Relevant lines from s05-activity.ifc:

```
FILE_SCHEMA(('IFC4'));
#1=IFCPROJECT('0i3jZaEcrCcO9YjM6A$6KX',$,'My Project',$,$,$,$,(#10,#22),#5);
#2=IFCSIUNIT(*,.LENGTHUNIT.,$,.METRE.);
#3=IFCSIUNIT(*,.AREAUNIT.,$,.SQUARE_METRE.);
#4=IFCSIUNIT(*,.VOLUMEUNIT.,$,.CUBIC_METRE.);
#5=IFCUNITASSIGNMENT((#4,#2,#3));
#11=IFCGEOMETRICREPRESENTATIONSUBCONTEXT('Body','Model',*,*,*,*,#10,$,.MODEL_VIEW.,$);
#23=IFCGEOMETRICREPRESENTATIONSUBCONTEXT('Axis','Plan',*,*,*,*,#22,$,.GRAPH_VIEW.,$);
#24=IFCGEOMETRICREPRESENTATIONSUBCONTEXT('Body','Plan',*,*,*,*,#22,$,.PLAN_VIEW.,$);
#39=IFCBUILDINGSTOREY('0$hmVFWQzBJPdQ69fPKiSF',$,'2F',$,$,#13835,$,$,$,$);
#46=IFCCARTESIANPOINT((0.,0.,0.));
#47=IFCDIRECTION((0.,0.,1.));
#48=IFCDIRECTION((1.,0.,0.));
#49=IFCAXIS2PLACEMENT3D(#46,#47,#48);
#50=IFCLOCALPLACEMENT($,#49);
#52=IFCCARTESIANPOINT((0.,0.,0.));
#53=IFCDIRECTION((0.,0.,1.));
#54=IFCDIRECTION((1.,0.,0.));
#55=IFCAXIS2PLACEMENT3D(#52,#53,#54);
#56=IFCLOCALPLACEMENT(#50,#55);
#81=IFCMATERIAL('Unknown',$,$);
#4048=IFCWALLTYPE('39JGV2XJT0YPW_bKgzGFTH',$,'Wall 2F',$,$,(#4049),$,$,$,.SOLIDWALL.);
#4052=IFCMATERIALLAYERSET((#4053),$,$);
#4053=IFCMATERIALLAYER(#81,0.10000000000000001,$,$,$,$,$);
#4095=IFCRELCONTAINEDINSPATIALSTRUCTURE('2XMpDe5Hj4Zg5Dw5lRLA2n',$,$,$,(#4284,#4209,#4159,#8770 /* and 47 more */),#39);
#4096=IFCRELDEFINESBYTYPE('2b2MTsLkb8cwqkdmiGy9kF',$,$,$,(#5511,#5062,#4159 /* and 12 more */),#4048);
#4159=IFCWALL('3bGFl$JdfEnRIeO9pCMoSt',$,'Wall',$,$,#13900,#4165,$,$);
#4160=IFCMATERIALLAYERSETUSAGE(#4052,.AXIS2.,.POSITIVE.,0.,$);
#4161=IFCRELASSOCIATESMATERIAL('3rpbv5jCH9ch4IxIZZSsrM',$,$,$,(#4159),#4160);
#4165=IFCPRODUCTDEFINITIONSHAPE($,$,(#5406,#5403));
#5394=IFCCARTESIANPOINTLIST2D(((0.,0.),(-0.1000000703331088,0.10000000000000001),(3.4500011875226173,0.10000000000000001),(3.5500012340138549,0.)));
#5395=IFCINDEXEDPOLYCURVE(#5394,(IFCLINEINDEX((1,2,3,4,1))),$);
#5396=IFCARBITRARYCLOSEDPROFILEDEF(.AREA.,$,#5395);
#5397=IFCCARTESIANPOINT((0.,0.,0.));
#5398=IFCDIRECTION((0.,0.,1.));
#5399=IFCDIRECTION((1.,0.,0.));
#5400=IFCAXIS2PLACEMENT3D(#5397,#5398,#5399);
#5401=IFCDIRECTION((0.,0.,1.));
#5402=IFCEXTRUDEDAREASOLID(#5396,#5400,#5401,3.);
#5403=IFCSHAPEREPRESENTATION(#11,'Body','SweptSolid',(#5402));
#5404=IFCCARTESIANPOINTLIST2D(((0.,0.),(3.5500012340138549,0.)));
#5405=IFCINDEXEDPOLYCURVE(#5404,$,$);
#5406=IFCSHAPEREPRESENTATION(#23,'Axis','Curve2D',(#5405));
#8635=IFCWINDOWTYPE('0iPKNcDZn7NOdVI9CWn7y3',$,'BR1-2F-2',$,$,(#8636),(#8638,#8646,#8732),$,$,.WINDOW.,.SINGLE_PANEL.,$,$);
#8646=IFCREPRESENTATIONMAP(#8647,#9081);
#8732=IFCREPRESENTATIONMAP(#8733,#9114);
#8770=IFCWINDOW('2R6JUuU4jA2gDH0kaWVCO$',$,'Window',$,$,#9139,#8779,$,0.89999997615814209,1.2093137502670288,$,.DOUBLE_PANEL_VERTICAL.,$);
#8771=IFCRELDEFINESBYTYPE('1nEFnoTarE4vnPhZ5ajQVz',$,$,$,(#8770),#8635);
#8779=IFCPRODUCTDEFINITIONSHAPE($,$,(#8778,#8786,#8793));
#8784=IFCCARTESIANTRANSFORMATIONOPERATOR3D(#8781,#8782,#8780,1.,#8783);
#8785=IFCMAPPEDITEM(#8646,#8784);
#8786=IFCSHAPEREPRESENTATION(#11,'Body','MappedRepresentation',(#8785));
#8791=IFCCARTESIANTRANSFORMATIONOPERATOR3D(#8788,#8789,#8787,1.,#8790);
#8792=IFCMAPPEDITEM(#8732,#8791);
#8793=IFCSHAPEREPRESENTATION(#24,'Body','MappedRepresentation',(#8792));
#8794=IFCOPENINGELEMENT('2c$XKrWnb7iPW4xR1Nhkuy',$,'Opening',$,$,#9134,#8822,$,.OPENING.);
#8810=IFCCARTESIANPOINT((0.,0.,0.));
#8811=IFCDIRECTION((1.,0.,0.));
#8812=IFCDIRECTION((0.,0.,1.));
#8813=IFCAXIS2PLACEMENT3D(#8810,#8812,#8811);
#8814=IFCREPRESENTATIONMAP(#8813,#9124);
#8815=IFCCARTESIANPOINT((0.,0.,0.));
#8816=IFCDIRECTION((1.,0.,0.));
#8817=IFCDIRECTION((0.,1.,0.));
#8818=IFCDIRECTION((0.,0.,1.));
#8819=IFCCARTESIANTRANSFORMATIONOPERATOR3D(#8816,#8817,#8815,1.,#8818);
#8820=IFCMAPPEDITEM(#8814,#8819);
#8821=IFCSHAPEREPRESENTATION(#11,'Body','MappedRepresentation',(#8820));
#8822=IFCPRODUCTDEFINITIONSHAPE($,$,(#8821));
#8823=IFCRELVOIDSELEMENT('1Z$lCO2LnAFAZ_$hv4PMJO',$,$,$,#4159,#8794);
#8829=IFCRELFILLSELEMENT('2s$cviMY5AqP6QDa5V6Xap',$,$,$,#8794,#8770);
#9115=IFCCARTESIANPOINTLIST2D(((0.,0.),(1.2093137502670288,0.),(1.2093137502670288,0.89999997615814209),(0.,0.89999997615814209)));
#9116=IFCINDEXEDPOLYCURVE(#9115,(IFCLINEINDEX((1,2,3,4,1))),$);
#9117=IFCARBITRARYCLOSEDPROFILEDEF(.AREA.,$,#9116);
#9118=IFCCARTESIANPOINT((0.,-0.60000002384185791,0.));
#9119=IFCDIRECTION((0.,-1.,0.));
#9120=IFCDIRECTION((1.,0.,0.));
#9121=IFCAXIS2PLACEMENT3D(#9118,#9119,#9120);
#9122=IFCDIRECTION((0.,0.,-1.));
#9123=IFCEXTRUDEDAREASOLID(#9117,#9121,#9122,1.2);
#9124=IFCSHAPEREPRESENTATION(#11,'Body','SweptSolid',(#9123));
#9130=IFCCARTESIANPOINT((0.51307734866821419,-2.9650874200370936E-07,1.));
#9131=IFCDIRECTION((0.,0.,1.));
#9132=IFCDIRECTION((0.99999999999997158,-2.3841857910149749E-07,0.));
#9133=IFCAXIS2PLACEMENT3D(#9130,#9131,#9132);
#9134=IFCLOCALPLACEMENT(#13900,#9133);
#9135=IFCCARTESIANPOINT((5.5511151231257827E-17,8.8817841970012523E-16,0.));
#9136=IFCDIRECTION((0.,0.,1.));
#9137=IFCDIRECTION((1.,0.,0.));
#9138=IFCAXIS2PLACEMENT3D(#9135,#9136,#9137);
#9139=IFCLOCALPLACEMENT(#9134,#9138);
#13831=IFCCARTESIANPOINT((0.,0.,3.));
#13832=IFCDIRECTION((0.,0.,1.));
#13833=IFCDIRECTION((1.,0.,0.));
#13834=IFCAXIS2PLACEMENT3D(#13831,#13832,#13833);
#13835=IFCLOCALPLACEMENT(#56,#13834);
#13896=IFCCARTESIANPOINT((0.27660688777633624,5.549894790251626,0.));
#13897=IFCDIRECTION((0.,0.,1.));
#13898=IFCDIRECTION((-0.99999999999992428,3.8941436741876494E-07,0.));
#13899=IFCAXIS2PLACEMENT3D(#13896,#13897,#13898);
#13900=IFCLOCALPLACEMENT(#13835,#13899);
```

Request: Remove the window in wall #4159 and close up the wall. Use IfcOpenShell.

```python
import ifcopenshell
import ifcopenshell.api.feature
import ifcopenshell.api.root
import ifcopenshell.geom
import ifcopenshell.util.shape

model = ifcopenshell.open("s05-activity.ifc")
settings = ifcopenshell.geom.settings()


def volume(element):
    """Net volume in cubic metres, openings subtracted."""
    shape = ifcopenshell.geom.create_shape(settings, element)
    return ifcopenshell.util.shape.get_volume(shape.geometry)


window = model.by_guid("2R6JUuU4jA2gDH0kaWVCO$")
opening = window.FillsVoids[0].RelatingOpeningElement
wall = opening.VoidsElements[0].RelatingBuildingElement
before = volume(wall)

ifcopenshell.api.root.remove_product(model, product=window)
ifcopenshell.api.feature.remove_feature(model, feature=opening)

after = volume(wall)

print(f"wall volume {before:.3f} -> {after:.3f} m3")

model.write("s05-activity-out.ifc")
```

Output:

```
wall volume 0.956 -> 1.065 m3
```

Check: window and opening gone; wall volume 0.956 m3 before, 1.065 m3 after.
